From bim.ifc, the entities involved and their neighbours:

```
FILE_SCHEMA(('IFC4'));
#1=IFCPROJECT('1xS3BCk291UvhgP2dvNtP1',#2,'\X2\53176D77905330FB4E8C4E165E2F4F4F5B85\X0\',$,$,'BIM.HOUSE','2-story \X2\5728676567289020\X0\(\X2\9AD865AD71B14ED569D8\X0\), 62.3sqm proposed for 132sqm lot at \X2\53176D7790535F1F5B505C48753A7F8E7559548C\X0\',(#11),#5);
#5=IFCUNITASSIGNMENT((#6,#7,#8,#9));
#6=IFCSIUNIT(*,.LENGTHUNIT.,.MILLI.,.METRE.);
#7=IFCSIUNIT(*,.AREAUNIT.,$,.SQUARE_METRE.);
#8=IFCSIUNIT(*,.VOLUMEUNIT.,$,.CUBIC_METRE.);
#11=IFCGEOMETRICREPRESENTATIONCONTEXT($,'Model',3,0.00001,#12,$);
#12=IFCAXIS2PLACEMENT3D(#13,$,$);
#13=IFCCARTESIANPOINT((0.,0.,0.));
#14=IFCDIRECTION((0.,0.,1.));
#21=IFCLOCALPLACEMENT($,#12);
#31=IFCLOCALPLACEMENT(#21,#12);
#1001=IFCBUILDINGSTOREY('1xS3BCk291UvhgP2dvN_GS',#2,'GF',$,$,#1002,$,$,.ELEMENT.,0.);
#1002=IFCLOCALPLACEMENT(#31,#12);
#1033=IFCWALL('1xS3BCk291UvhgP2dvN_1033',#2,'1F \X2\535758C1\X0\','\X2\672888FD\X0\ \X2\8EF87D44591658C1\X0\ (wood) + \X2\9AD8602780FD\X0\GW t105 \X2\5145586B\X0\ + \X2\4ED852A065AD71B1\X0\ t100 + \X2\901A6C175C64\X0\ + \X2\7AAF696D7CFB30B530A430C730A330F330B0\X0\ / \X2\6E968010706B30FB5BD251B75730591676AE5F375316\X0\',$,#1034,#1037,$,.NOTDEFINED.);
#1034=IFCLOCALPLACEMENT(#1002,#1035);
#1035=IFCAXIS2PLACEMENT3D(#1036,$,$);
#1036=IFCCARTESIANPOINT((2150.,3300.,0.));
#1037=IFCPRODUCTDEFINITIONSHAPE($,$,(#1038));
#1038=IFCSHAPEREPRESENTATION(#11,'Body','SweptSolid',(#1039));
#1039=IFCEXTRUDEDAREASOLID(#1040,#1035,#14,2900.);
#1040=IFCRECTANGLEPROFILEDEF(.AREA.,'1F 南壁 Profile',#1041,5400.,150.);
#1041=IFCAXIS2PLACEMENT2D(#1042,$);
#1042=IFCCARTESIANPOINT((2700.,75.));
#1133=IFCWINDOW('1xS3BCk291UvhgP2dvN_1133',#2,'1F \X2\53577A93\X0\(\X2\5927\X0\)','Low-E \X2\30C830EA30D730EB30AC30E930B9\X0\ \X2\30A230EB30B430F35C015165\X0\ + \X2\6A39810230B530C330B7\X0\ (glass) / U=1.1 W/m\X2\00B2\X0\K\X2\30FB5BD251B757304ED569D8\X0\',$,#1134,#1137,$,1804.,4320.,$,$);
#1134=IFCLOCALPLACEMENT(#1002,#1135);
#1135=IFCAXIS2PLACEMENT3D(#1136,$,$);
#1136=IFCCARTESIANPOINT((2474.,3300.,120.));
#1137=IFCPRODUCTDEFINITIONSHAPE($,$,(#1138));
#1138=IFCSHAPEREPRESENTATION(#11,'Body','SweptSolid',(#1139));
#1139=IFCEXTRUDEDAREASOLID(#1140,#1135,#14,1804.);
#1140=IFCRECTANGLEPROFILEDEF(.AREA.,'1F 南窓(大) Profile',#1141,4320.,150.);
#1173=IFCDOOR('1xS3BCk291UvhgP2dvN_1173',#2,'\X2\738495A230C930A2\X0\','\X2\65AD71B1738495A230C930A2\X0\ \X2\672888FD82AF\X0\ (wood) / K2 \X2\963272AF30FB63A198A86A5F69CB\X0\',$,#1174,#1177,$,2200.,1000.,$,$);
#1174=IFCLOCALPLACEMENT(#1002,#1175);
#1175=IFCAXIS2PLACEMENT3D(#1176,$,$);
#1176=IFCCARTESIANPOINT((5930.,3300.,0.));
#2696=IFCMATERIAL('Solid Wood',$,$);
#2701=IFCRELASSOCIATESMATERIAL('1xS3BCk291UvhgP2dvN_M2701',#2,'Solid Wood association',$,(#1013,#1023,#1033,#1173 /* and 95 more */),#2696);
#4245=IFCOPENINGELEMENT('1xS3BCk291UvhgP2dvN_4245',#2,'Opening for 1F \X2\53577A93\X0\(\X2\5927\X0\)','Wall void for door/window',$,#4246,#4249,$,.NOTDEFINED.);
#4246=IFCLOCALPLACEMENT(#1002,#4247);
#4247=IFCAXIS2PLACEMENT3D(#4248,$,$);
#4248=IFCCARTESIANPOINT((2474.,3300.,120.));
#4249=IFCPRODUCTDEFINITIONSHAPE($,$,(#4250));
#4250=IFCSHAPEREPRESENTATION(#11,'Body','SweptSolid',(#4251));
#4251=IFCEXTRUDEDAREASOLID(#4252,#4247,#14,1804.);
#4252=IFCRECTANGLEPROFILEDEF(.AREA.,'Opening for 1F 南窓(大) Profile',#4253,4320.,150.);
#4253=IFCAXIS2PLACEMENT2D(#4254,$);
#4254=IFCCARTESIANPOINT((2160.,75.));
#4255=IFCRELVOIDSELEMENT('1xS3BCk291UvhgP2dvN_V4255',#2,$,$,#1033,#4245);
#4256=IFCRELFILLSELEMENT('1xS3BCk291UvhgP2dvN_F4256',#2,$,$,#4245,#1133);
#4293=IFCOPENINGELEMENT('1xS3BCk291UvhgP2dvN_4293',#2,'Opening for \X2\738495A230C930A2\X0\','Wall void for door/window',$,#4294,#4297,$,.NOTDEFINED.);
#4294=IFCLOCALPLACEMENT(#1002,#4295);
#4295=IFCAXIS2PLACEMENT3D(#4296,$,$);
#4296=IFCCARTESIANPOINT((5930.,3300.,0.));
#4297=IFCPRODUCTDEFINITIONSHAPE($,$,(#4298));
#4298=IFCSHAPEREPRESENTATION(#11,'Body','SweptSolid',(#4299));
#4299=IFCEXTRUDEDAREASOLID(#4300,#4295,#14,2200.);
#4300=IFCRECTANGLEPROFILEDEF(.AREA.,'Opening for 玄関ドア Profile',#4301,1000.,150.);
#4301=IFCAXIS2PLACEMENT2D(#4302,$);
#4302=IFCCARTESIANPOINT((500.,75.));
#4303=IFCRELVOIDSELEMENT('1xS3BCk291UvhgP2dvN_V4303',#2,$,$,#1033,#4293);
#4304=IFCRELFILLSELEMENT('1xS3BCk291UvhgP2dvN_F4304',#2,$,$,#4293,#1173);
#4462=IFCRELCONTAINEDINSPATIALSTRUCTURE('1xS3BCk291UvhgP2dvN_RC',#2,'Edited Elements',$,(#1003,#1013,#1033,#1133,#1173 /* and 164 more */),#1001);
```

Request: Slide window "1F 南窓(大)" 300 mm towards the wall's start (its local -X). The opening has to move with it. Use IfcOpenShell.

```python
import ifcopenshell
import ifcopenshell.api.geometry
import ifcopenshell.util.placement
import ifcopenshell.util.unit

model = ifcopenshell.open("bim.ifc")
unit_scale = ifcopenshell.util.unit.calculate_unit_scale(model)

window = model.by_guid("1xS3BCk291UvhgP2dvN_1133")
opening = window.FillsVoids[0].RelatingOpeningElement
wall = opening.VoidsElements[0].RelatingBuildingElement

wall_matrix = ifcopenshell.util.placement.get_local_placement(wall.ObjectPlacement)
shift = wall_matrix[:3, 0] * -0.3 / unit_scale
before = ifcopenshell.util.placement.get_local_placement(window.ObjectPlacement)[:3, 3].copy()

# The window is not placed relative to its opening, so move both.
for product in (opening, window):
    matrix = ifcopenshell.util.placement.get_local_placement(product.ObjectPlacement)
    matrix[:3, 3] += shift
    ifcopenshell.api.geometry.edit_object_placement(model, product=product, matrix=matrix, is_si=False)

after = ifcopenshell.util.placement.get_local_placement(window.ObjectPlacement)[:3, 3]
print("window moved by", (after - before).round(3) + 0.0)

model.write("bim-out.ifc")
```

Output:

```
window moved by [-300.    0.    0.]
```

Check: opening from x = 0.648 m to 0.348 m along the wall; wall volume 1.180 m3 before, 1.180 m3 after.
